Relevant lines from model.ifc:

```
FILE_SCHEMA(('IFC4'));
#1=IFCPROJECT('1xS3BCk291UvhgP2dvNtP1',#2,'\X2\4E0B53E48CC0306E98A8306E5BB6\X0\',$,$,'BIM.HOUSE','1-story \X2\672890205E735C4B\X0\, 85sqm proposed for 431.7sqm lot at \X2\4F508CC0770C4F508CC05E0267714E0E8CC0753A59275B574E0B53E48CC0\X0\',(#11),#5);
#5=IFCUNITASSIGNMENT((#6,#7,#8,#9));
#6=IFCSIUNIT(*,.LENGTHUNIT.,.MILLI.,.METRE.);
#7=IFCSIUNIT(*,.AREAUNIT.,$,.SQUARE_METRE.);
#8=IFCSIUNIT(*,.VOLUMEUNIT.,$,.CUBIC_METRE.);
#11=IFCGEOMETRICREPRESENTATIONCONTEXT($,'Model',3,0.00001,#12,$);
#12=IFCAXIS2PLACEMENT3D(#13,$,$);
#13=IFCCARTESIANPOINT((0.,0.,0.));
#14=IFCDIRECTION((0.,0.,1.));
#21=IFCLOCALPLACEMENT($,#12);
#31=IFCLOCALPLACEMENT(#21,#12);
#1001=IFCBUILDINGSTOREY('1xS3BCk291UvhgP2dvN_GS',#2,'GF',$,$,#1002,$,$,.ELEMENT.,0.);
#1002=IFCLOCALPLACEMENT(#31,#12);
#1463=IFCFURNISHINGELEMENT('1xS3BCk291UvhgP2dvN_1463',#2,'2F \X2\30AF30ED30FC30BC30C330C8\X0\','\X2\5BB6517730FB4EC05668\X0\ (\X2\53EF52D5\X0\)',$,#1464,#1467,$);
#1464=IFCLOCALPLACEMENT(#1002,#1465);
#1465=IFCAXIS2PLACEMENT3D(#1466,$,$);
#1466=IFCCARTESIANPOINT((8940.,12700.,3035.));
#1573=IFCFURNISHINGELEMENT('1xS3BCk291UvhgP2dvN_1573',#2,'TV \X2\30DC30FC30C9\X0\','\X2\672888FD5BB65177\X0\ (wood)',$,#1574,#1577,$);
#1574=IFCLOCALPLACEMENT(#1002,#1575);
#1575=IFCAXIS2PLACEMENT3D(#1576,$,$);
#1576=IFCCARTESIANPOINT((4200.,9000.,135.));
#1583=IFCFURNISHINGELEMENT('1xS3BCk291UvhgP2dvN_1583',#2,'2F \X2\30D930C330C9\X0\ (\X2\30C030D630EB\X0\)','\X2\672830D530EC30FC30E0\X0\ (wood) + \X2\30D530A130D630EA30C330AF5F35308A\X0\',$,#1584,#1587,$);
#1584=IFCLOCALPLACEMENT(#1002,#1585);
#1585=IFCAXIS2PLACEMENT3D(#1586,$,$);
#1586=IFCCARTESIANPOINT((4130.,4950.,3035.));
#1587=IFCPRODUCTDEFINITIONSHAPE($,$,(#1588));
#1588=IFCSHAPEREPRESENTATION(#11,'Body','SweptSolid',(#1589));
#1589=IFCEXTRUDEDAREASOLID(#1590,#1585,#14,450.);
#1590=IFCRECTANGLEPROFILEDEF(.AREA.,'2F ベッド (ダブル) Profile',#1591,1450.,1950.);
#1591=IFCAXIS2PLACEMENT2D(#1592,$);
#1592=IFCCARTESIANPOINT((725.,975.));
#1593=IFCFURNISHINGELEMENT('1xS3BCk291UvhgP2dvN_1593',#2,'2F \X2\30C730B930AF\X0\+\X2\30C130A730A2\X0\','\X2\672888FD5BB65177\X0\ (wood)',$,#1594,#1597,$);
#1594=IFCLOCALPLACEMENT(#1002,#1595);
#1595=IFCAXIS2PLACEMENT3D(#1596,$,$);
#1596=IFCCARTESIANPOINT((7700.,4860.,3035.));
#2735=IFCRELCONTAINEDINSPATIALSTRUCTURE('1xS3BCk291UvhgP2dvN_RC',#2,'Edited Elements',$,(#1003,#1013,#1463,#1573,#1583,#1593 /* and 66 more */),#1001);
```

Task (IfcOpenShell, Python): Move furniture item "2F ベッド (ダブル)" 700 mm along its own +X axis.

```python
import ifcopenshell
import ifcopenshell.api.geometry
import ifcopenshell.util.placement
import ifcopenshell.util.unit

model = ifcopenshell.open("model.ifc")
unit_scale = ifcopenshell.util.unit.calculate_unit_scale(model)

item = model.by_guid("1xS3BCk291UvhgP2dvN_1583")
matrix = ifcopenshell.util.placement.get_local_placement(item.ObjectPlacement)
matrix[:3, 3] += matrix[:3, 0] * 0.7 / unit_scale
ifcopenshell.api.geometry.edit_object_placement(model, product=item, matrix=matrix, is_si=False)

print(ifcopenshell.util.placement.get_local_placement(item.ObjectPlacement).round(3) + 0.0)

model.write("model_updated.ifc")
```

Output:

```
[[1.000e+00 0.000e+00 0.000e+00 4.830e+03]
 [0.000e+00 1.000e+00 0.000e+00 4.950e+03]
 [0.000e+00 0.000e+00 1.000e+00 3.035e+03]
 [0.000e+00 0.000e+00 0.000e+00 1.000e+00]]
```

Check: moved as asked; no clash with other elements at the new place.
